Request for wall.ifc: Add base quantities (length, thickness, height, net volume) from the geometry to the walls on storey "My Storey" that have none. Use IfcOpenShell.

First a look at what the model holds.

```python
import ifcopenshell
import ifcopenshell.util.element
import ifcopenshell.util.unit

model = ifcopenshell.open("wall.ifc")
print(model.schema)
for unit_type in ("LENGTHUNIT", "AREAUNIT", "VOLUMEUNIT"):
    print(unit_type, ifcopenshell.util.unit.calculate_unit_scale(model, unit_type))
storey = next(s for s in model.by_type("IfcBuildingStorey") if s.Name == "My Storey")
walls = [e for e in ifcopenshell.util.element.get_decomposition(storey) if e.is_a("IfcWall")]
for e in sorted(walls, key=lambda e: e.id()):
    print(e.id(), e.is_a(), e.Name, list(ifcopenshell.util.element.get_psets(e, qtos_only=True)), sep=" | ")
```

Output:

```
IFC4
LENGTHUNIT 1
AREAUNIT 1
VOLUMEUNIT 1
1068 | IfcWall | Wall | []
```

```python
import ifcopenshell
import ifcopenshell.api.pset
import ifcopenshell.geom
import ifcopenshell.util.element
import ifcopenshell.util.shape
import ifcopenshell.util.unit

model = ifcopenshell.open("wall.ifc")
unit_scale = ifcopenshell.util.unit.calculate_unit_scale(model)
volume_scale = ifcopenshell.util.unit.calculate_unit_scale(model, "VOLUMEUNIT")
settings = ifcopenshell.geom.settings()

storey = next(s for s in model.by_type("IfcBuildingStorey") if s.Name == "My Storey")
walls = [e for e in ifcopenshell.util.element.get_decomposition(storey) if e.is_a("IfcWall")]

for e in sorted(walls, key=lambda e: e.id()):
    if ifcopenshell.util.element.get_psets(e, qtos_only=True, should_inherit=False):
        continue
    # Geometry comes back in metres, in the element's own axes.
    shape = ifcopenshell.geom.create_shape(settings, e)
    values = {
        "Length": ifcopenshell.util.shape.get_x(shape.geometry) / unit_scale,
        "Width": ifcopenshell.util.shape.get_y(shape.geometry) / unit_scale,
        "Height": ifcopenshell.util.shape.get_z(shape.geometry) / unit_scale,
        "NetVolume": ifcopenshell.util.shape.get_volume(shape.geometry) / volume_scale,
    }
    qto = ifcopenshell.api.pset.add_qto(model, product=e, name="Qto_WallBaseQuantities")
    ifcopenshell.api.pset.edit_qto(model, qto=qto, properties=values)
    print(e.id(), {k: round(v, 3) for k, v in values.items()})

model.write("wall_updated.ifc")
```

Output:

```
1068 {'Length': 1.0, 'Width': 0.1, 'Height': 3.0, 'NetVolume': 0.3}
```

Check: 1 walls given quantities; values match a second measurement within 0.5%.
